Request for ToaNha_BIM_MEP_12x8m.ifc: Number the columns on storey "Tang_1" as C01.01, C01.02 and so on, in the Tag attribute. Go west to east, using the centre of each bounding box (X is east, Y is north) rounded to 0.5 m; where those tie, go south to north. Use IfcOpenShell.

First a look at what the model holds.

```python
import ifcopenshell
import ifcopenshell.util.element
import ifcopenshell.util.placement

model = ifcopenshell.open("ToaNha_BIM_MEP_12x8m.ifc")
print(model.schema)
storey = next(s for s in model.by_type("IfcBuildingStorey") if s.Name == "Tang_1")
columns = [e for e in ifcopenshell.util.element.get_decomposition(storey) if e.is_a("IfcColumn")]
for e in sorted(columns, key=lambda e: e.id()):
    origin = ifcopenshell.util.placement.get_local_placement(e.ObjectPlacement)[:3, 3]
    print(e.id(), e.Tag, e.Name, origin.round(2) + 0.0, sep=" | ")
```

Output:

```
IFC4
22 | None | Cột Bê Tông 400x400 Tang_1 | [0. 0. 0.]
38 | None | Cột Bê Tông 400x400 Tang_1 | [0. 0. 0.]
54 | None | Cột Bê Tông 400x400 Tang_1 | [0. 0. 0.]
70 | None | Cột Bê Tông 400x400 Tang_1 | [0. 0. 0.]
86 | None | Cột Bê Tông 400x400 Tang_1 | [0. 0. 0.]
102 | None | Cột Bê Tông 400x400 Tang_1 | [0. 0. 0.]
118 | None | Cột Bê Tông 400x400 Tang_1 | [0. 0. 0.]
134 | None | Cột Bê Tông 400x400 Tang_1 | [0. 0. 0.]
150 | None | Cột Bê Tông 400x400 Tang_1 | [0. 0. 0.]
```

```python
import ifcopenshell
import ifcopenshell.geom
import ifcopenshell.util.element
import ifcopenshell.util.shape

model = ifcopenshell.open("ToaNha_BIM_MEP_12x8m.ifc")
settings = ifcopenshell.geom.settings()
settings.set("use-world-coords", True)


def centre(element):
    shape = ifcopenshell.geom.create_shape(settings, element)
    return ifcopenshell.util.shape.get_bbox_centroid(shape.geometry)


storey = next(s for s in model.by_type("IfcBuildingStorey") if s.Name == "Tang_1")
columns = [e for e in ifcopenshell.util.element.get_decomposition(storey) if e.is_a("IfcColumn")]

# Insertion points can sit at a corner or the storey origin, so sort by the geometry (in metres).
centres = {e: centre(e) for e in columns}
columns.sort(key=lambda e: (round(centres[e][0] / 0.5), centres[e][1]))

for i, e in enumerate(columns, start=1):
    number = f"C01.{i:02d}"
    e.Tag = number
    print(e.id(), number)

model.write("ToaNha_BIM_MEP_12x8m-out.ifc")
```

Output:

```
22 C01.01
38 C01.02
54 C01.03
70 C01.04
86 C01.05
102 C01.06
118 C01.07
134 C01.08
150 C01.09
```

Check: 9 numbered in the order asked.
